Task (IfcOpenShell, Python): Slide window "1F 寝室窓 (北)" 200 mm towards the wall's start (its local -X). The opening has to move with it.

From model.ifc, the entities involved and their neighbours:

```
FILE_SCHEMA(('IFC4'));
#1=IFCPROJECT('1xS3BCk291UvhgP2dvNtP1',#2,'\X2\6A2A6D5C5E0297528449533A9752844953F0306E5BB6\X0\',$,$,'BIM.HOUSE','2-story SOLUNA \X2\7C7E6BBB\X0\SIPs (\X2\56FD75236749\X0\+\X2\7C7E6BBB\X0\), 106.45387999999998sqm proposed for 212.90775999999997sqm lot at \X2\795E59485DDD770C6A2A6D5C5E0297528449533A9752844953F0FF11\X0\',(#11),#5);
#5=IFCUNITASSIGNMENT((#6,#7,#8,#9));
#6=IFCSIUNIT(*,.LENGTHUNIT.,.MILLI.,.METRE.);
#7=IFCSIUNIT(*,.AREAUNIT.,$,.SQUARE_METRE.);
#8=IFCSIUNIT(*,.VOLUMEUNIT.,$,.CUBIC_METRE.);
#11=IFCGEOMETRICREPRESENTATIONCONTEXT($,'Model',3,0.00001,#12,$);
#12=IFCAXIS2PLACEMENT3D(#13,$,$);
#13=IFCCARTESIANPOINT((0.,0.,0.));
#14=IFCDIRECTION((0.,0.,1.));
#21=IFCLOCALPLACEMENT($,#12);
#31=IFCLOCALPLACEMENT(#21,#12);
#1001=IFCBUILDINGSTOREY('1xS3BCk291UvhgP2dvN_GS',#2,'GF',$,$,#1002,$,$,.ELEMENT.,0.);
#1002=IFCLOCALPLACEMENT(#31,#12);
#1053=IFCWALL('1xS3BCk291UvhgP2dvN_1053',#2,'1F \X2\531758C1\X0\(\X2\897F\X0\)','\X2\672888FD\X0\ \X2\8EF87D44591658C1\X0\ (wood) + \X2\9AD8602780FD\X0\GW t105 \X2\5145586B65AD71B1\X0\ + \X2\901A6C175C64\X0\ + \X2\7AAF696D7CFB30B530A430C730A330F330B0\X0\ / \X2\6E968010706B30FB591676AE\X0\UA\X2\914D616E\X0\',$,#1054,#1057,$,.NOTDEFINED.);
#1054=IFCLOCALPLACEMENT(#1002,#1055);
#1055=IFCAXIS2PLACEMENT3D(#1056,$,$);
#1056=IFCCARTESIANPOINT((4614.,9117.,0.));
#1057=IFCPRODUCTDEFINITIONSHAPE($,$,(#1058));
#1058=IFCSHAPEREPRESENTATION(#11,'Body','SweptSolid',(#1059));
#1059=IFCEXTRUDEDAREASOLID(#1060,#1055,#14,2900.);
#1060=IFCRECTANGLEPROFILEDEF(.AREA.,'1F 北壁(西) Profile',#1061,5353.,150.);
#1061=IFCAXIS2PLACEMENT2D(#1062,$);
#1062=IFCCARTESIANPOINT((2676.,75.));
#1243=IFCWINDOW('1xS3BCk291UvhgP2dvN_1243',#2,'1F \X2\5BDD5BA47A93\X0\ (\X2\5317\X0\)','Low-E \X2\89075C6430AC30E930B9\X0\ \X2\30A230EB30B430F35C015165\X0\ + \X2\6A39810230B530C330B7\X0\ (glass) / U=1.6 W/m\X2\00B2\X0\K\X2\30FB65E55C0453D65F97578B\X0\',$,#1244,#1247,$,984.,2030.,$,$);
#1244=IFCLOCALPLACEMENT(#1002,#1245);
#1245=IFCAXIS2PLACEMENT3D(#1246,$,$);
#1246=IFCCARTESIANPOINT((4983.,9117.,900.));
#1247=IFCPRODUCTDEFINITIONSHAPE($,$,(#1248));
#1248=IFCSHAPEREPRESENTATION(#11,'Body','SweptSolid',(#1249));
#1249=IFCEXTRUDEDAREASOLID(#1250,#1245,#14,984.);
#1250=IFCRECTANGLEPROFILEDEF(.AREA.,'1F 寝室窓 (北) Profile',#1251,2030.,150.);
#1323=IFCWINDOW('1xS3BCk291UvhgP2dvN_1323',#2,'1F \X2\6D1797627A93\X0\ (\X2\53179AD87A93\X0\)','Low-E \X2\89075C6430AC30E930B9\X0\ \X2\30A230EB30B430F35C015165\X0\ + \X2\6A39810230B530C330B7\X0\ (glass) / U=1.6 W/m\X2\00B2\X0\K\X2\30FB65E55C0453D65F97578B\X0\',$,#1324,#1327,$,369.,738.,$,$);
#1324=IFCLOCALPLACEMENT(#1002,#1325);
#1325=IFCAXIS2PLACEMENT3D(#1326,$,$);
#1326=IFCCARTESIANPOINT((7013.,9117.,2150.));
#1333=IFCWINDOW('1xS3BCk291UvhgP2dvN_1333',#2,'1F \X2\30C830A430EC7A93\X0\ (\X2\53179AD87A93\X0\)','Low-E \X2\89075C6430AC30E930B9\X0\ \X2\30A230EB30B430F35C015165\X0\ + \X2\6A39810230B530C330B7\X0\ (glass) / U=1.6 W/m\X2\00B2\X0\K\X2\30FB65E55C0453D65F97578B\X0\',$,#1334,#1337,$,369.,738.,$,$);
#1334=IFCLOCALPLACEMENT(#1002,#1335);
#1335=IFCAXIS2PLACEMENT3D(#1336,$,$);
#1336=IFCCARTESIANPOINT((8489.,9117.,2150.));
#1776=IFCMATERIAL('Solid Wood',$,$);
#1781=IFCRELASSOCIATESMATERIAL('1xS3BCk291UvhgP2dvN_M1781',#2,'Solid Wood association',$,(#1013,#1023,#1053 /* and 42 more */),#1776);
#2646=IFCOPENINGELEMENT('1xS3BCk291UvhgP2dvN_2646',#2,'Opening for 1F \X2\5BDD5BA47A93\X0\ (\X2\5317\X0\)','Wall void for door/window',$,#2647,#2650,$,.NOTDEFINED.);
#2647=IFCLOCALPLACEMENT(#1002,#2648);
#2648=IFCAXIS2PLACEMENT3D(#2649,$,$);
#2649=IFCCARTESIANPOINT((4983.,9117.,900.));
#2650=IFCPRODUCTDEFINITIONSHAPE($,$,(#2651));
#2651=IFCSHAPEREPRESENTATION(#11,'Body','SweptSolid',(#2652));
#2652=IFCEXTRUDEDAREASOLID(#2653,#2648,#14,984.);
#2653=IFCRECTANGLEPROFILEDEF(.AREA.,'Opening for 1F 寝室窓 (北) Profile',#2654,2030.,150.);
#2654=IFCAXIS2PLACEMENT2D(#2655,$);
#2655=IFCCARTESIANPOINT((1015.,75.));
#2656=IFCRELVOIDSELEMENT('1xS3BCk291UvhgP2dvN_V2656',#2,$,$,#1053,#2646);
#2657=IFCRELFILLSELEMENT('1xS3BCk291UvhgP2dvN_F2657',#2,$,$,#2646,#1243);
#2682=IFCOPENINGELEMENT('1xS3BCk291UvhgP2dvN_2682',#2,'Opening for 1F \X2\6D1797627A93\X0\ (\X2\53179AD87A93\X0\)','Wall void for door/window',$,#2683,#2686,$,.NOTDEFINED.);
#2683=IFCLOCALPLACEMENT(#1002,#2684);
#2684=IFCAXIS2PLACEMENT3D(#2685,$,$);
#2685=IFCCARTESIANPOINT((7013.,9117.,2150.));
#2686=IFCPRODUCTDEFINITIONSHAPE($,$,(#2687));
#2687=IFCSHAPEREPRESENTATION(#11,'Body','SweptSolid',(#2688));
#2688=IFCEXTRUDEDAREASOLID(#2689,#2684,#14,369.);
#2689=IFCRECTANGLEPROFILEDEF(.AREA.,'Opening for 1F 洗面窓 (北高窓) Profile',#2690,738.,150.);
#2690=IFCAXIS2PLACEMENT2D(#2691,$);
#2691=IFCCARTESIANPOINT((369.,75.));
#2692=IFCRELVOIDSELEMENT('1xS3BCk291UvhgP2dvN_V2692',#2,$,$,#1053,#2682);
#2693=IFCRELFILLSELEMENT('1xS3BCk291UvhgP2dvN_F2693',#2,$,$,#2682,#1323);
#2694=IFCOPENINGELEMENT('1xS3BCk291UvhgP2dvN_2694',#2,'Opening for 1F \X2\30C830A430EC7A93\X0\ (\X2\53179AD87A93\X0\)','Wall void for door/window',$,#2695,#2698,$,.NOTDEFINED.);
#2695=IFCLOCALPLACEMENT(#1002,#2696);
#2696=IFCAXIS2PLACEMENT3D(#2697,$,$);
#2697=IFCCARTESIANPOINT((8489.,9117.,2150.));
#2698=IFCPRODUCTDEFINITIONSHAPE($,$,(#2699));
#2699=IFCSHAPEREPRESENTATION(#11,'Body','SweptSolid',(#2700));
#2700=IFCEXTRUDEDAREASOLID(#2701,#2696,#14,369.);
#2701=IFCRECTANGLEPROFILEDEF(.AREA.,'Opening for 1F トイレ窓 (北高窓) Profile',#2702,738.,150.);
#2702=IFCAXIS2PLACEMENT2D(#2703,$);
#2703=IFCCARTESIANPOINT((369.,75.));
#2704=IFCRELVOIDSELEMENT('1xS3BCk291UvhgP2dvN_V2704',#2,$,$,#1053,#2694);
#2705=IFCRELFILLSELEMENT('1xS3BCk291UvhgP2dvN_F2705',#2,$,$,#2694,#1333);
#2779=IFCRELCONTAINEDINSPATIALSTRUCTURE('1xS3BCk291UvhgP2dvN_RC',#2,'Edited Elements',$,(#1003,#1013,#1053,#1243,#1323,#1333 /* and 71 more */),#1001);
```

```python
import ifcopenshell
import ifcopenshell.api.geometry
import ifcopenshell.util.placement

model = ifcopenshell.open("model.ifc")

window = model.by_guid("1xS3BCk291UvhgP2dvN_1243")
opening = window.FillsVoids[0].RelatingOpeningElement
wall = opening.VoidsElements[0].RelatingBuildingElement

wall_matrix = ifcopenshell.util.placement.get_local_placement(wall.ObjectPlacement)
shift = wall_matrix[:3, 0] * -200.0
before = ifcopenshell.util.placement.get_local_placement(window.ObjectPlacement)[:3, 3].copy()

# The window is not placed relative to its opening, so move both.
for product in (opening, window):
    matrix = ifcopenshell.util.placement.get_local_placement(product.ObjectPlacement)
    matrix[:3, 3] += shift
    ifcopenshell.api.geometry.edit_object_placement(model, product=product, matrix=matrix, is_si=False)

after = ifcopenshell.util.placement.get_local_placement(window.ObjectPlacement)[:3, 3]
print("window moved by", (after - before).round(3) + 0.0)

model.write("model_updated.ifc")
```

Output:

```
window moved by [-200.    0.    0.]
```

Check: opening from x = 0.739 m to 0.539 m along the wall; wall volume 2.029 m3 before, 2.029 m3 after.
